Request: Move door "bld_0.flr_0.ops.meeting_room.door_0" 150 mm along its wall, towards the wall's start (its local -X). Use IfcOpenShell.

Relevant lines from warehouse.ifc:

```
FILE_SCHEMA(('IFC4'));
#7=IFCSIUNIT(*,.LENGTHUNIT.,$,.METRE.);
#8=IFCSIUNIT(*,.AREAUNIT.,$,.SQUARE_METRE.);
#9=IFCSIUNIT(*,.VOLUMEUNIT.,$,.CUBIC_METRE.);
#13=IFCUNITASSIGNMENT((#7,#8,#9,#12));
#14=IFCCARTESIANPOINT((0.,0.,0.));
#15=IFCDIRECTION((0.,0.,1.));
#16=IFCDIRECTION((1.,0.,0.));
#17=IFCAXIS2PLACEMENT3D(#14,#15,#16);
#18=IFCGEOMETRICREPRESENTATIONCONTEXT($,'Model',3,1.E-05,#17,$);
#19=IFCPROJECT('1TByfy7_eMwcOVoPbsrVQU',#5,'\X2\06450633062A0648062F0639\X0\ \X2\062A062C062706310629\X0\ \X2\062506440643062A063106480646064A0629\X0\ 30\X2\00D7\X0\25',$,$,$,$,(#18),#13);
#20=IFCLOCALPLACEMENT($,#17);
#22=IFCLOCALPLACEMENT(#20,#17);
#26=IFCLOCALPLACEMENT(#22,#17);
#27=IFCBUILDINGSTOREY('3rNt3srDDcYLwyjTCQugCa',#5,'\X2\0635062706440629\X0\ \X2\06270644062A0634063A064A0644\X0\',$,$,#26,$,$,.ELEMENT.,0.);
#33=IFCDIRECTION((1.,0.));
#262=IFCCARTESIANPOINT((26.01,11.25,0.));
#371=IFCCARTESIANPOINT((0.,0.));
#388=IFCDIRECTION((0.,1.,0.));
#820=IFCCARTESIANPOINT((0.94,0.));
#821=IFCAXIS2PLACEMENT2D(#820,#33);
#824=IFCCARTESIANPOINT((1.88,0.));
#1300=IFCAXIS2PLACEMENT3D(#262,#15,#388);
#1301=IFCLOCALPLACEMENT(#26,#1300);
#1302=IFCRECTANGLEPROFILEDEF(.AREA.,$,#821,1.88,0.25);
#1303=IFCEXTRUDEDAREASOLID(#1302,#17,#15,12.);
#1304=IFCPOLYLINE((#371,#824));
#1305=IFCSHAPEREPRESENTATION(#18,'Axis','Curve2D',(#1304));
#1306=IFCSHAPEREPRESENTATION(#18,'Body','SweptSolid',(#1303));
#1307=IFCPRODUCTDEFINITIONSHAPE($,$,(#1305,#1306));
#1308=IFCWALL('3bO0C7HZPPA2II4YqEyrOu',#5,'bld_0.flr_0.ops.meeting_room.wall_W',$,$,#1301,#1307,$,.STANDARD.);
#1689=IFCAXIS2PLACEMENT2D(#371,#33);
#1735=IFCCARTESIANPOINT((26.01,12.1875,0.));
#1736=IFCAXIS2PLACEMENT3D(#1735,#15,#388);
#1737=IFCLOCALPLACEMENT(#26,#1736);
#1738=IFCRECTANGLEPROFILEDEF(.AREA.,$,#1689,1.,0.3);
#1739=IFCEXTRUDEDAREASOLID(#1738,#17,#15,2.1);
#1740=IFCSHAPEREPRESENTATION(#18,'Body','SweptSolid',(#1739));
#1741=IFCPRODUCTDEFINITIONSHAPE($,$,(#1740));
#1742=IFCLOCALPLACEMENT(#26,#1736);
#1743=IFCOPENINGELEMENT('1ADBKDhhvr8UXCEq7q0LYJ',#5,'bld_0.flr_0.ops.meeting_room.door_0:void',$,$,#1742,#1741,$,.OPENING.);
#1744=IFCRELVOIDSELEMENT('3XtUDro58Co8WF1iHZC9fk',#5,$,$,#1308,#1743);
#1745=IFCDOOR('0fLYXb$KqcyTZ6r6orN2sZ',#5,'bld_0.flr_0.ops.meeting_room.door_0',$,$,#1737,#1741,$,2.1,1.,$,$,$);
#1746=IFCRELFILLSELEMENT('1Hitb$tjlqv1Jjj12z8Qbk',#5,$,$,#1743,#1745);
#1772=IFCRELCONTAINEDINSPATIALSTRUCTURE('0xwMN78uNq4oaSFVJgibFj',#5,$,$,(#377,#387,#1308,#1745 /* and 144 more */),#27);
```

```python
import ifcopenshell
import ifcopenshell.api.geometry
import ifcopenshell.util.placement
import ifcopenshell.util.unit

model = ifcopenshell.open("warehouse.ifc")
unit_scale = ifcopenshell.util.unit.calculate_unit_scale(model)

door = model.by_guid("0fLYXb$KqcyTZ6r6orN2sZ")
opening = door.FillsVoids[0].RelatingOpeningElement
wall = opening.VoidsElements[0].RelatingBuildingElement

wall_matrix = ifcopenshell.util.placement.get_local_placement(wall.ObjectPlacement)
shift = wall_matrix[:3, 0] * -0.15 / unit_scale
before = ifcopenshell.util.placement.get_local_placement(door.ObjectPlacement)[:3, 3].copy()

# The door is not placed relative to its opening, so move both.
for product in (opening, door):
    matrix = ifcopenshell.util.placement.get_local_placement(product.ObjectPlacement)
    matrix[:3, 3] += shift
    ifcopenshell.api.geometry.edit_object_placement(model, product=product, matrix=matrix, is_si=False)

after = ifcopenshell.util.placement.get_local_placement(door.ObjectPlacement)[:3, 3]
print("door moved by", (after - before).round(3) + 0.0)

model.write("warehouse_updated.ifc")
```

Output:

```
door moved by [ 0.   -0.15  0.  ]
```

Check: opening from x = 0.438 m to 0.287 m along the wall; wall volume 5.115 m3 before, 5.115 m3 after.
